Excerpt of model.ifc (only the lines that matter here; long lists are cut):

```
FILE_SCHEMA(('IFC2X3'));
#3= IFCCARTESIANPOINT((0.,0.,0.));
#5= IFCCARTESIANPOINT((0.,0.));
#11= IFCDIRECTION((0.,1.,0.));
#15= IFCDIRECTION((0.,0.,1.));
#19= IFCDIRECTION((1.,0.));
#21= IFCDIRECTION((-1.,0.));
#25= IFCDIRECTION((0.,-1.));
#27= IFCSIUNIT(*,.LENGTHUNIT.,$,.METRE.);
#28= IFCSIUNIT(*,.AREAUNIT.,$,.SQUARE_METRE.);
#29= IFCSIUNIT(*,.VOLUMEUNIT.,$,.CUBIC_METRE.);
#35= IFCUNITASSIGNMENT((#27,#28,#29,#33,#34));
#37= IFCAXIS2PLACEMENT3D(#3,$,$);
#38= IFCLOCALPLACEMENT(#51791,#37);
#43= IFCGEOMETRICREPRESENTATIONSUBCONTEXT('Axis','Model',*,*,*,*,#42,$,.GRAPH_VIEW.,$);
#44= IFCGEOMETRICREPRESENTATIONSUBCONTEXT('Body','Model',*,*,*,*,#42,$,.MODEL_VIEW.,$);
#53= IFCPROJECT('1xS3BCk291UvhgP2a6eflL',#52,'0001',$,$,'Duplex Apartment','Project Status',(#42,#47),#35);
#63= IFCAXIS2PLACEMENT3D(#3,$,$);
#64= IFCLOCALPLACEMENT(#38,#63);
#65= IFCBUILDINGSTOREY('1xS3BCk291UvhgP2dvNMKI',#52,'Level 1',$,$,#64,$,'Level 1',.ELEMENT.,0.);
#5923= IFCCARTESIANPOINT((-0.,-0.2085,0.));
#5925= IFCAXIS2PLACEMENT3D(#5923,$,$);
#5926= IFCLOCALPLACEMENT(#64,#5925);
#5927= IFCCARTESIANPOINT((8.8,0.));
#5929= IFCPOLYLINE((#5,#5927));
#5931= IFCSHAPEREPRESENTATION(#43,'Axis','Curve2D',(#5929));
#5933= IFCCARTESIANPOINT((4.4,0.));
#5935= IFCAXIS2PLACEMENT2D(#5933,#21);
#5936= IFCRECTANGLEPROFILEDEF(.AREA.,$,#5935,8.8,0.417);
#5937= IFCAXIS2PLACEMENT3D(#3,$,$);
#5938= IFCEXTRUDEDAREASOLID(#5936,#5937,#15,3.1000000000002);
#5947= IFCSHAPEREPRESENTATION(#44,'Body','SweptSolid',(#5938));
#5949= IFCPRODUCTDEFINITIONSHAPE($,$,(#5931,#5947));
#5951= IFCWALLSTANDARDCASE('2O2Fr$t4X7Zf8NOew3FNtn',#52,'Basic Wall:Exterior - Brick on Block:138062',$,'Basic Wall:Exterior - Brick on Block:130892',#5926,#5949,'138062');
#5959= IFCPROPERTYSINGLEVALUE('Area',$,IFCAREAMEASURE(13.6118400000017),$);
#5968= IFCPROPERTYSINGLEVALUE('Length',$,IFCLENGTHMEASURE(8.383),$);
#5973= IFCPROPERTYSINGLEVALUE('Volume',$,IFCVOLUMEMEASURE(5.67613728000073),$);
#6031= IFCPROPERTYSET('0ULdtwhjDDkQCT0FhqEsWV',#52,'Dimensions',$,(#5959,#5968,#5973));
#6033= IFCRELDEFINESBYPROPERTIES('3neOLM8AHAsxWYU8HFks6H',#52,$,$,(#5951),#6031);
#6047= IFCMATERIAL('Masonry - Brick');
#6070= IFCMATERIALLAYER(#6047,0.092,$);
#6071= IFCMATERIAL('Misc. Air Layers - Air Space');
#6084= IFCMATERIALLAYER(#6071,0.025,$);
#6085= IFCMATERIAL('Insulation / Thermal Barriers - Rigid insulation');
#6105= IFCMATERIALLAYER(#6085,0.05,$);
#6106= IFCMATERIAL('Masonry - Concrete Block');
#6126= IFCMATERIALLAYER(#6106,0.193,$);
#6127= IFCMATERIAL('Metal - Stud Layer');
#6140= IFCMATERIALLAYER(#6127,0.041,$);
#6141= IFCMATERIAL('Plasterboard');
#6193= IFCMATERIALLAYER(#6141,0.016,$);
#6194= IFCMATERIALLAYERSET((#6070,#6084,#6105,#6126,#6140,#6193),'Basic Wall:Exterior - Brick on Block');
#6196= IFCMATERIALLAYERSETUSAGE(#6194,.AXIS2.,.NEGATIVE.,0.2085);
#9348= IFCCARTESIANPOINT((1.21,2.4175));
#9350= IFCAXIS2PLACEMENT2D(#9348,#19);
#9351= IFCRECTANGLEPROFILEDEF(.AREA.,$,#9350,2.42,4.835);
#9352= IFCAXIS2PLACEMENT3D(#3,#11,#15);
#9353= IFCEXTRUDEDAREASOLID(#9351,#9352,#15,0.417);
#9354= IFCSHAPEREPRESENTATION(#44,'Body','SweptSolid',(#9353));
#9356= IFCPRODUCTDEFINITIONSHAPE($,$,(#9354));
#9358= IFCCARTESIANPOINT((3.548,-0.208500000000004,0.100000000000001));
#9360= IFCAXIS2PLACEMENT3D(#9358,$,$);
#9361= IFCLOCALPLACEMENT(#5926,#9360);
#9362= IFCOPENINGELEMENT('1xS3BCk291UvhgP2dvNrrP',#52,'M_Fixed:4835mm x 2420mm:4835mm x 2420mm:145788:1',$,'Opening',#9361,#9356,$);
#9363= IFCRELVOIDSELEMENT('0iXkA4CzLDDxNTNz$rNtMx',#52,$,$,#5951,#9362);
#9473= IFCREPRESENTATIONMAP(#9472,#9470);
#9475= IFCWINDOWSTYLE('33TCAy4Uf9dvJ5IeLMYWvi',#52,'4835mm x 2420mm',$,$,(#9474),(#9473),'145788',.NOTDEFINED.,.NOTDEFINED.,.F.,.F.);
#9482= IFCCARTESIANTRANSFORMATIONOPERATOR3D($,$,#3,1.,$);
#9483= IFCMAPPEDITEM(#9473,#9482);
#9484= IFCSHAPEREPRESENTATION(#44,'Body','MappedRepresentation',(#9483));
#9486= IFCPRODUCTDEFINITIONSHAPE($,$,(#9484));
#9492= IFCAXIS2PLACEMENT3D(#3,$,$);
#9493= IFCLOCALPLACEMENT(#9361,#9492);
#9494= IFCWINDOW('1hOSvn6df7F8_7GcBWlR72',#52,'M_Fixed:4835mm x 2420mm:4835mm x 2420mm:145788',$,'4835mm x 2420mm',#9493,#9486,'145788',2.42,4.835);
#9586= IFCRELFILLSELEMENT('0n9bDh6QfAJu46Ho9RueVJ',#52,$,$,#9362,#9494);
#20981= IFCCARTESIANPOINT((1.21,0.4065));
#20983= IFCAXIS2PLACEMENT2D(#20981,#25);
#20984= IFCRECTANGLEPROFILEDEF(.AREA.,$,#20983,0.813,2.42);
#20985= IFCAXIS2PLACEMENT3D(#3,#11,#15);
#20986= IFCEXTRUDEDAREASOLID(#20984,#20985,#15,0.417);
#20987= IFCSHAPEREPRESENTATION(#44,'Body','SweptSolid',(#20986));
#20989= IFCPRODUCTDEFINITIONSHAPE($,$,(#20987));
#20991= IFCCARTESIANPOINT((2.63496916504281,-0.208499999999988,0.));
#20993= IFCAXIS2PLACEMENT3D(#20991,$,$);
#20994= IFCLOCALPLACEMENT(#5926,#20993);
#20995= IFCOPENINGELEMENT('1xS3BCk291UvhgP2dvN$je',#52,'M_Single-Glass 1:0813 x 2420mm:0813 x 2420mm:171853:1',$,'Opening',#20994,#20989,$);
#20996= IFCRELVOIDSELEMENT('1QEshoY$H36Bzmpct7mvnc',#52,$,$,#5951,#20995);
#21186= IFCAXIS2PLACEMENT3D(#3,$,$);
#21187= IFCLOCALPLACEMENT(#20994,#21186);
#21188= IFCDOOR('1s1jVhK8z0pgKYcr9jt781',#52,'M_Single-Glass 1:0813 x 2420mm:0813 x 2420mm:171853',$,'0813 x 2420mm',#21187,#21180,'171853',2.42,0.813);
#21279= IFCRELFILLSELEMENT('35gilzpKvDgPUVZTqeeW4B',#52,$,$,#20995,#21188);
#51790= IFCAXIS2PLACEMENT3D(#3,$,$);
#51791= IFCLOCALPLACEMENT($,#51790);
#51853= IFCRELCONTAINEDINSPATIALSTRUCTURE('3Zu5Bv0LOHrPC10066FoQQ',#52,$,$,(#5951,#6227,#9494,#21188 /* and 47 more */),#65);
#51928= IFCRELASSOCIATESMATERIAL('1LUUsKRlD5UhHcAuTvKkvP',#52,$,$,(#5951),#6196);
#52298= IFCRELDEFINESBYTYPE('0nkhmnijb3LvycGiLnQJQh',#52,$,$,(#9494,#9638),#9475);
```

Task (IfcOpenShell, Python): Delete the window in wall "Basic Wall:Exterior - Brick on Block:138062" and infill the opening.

```python
import ifcopenshell
import ifcopenshell.api.feature
import ifcopenshell.api.pset
import ifcopenshell.api.root
import ifcopenshell.geom
import ifcopenshell.util.element
import ifcopenshell.util.shape
import ifcopenshell.util.unit

model = ifcopenshell.open("model.ifc")
area_scale = ifcopenshell.util.unit.calculate_unit_scale(model, "AREAUNIT")
volume_scale = ifcopenshell.util.unit.calculate_unit_scale(model, "VOLUMEUNIT")
settings = ifcopenshell.geom.settings()


def volume(element):
    """Net volume in cubic metres, openings subtracted."""
    shape = ifcopenshell.geom.create_shape(settings, element)
    return ifcopenshell.util.shape.get_volume(shape.geometry)


window = model.by_guid("1hOSvn6df7F8_7GcBWlR72")
opening = window.FillsVoids[0].RelatingOpeningElement
wall = opening.VoidsElements[0].RelatingBuildingElement
before = volume(wall)

ifcopenshell.api.root.remove_product(model, product=window)
ifcopenshell.api.feature.remove_feature(model, feature=opening)

after = volume(wall)
thickness = 0.417  # wall thickness in metres

# Update the wall's stored quantities.
pset = model.by_id(ifcopenshell.util.element.get_pset(wall, "Dimensions", should_inherit=False)["id"])
ifcopenshell.api.pset.edit_pset(model, pset=pset, properties={
    "Area": model.create_entity("IfcAreaMeasure", after / thickness / area_scale),
    "Volume": model.create_entity("IfcVolumeMeasure", after / volume_scale),
})

print(f"wall volume {before:.3f} -> {after:.3f} m3")

model.write("model_edited.ifc")
```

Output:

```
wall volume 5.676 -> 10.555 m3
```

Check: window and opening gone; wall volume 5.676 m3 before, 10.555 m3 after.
